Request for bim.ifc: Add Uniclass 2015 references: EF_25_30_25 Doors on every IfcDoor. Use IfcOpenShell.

First a look at what the model holds.

```python
import ifcopenshell

model = ifcopenshell.open("bim.ifc")
print(model.schema)
print("classifications:", [c.Name for c in model.by_type("IfcClassification")])
for ifc_class in ("IfcDoor", "IfcRoof", "IfcStair", "IfcWall", "IfcWindow"):
    print(ifc_class, len(model.by_type(ifc_class)))
```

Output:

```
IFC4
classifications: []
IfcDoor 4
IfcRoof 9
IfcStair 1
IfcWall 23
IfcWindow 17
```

```python
import ifcopenshell
import ifcopenshell.api.classification

model = ifcopenshell.open("bim.ifc")

system = ifcopenshell.api.classification.add_classification(model, classification="Uniclass 2015")

codes = {
    "IfcDoor": ("EF_25_30_25", "Doors"),
}
for ifc_class, (code, name) in codes.items():
    products = model.by_type(ifc_class)
    ifcopenshell.api.classification.add_reference(
        model, products=products, classification=system, identification=code, name=name
    )
    print(code, len(products))

model.write("bim_rev.ifc")
```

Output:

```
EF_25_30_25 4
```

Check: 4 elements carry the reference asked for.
